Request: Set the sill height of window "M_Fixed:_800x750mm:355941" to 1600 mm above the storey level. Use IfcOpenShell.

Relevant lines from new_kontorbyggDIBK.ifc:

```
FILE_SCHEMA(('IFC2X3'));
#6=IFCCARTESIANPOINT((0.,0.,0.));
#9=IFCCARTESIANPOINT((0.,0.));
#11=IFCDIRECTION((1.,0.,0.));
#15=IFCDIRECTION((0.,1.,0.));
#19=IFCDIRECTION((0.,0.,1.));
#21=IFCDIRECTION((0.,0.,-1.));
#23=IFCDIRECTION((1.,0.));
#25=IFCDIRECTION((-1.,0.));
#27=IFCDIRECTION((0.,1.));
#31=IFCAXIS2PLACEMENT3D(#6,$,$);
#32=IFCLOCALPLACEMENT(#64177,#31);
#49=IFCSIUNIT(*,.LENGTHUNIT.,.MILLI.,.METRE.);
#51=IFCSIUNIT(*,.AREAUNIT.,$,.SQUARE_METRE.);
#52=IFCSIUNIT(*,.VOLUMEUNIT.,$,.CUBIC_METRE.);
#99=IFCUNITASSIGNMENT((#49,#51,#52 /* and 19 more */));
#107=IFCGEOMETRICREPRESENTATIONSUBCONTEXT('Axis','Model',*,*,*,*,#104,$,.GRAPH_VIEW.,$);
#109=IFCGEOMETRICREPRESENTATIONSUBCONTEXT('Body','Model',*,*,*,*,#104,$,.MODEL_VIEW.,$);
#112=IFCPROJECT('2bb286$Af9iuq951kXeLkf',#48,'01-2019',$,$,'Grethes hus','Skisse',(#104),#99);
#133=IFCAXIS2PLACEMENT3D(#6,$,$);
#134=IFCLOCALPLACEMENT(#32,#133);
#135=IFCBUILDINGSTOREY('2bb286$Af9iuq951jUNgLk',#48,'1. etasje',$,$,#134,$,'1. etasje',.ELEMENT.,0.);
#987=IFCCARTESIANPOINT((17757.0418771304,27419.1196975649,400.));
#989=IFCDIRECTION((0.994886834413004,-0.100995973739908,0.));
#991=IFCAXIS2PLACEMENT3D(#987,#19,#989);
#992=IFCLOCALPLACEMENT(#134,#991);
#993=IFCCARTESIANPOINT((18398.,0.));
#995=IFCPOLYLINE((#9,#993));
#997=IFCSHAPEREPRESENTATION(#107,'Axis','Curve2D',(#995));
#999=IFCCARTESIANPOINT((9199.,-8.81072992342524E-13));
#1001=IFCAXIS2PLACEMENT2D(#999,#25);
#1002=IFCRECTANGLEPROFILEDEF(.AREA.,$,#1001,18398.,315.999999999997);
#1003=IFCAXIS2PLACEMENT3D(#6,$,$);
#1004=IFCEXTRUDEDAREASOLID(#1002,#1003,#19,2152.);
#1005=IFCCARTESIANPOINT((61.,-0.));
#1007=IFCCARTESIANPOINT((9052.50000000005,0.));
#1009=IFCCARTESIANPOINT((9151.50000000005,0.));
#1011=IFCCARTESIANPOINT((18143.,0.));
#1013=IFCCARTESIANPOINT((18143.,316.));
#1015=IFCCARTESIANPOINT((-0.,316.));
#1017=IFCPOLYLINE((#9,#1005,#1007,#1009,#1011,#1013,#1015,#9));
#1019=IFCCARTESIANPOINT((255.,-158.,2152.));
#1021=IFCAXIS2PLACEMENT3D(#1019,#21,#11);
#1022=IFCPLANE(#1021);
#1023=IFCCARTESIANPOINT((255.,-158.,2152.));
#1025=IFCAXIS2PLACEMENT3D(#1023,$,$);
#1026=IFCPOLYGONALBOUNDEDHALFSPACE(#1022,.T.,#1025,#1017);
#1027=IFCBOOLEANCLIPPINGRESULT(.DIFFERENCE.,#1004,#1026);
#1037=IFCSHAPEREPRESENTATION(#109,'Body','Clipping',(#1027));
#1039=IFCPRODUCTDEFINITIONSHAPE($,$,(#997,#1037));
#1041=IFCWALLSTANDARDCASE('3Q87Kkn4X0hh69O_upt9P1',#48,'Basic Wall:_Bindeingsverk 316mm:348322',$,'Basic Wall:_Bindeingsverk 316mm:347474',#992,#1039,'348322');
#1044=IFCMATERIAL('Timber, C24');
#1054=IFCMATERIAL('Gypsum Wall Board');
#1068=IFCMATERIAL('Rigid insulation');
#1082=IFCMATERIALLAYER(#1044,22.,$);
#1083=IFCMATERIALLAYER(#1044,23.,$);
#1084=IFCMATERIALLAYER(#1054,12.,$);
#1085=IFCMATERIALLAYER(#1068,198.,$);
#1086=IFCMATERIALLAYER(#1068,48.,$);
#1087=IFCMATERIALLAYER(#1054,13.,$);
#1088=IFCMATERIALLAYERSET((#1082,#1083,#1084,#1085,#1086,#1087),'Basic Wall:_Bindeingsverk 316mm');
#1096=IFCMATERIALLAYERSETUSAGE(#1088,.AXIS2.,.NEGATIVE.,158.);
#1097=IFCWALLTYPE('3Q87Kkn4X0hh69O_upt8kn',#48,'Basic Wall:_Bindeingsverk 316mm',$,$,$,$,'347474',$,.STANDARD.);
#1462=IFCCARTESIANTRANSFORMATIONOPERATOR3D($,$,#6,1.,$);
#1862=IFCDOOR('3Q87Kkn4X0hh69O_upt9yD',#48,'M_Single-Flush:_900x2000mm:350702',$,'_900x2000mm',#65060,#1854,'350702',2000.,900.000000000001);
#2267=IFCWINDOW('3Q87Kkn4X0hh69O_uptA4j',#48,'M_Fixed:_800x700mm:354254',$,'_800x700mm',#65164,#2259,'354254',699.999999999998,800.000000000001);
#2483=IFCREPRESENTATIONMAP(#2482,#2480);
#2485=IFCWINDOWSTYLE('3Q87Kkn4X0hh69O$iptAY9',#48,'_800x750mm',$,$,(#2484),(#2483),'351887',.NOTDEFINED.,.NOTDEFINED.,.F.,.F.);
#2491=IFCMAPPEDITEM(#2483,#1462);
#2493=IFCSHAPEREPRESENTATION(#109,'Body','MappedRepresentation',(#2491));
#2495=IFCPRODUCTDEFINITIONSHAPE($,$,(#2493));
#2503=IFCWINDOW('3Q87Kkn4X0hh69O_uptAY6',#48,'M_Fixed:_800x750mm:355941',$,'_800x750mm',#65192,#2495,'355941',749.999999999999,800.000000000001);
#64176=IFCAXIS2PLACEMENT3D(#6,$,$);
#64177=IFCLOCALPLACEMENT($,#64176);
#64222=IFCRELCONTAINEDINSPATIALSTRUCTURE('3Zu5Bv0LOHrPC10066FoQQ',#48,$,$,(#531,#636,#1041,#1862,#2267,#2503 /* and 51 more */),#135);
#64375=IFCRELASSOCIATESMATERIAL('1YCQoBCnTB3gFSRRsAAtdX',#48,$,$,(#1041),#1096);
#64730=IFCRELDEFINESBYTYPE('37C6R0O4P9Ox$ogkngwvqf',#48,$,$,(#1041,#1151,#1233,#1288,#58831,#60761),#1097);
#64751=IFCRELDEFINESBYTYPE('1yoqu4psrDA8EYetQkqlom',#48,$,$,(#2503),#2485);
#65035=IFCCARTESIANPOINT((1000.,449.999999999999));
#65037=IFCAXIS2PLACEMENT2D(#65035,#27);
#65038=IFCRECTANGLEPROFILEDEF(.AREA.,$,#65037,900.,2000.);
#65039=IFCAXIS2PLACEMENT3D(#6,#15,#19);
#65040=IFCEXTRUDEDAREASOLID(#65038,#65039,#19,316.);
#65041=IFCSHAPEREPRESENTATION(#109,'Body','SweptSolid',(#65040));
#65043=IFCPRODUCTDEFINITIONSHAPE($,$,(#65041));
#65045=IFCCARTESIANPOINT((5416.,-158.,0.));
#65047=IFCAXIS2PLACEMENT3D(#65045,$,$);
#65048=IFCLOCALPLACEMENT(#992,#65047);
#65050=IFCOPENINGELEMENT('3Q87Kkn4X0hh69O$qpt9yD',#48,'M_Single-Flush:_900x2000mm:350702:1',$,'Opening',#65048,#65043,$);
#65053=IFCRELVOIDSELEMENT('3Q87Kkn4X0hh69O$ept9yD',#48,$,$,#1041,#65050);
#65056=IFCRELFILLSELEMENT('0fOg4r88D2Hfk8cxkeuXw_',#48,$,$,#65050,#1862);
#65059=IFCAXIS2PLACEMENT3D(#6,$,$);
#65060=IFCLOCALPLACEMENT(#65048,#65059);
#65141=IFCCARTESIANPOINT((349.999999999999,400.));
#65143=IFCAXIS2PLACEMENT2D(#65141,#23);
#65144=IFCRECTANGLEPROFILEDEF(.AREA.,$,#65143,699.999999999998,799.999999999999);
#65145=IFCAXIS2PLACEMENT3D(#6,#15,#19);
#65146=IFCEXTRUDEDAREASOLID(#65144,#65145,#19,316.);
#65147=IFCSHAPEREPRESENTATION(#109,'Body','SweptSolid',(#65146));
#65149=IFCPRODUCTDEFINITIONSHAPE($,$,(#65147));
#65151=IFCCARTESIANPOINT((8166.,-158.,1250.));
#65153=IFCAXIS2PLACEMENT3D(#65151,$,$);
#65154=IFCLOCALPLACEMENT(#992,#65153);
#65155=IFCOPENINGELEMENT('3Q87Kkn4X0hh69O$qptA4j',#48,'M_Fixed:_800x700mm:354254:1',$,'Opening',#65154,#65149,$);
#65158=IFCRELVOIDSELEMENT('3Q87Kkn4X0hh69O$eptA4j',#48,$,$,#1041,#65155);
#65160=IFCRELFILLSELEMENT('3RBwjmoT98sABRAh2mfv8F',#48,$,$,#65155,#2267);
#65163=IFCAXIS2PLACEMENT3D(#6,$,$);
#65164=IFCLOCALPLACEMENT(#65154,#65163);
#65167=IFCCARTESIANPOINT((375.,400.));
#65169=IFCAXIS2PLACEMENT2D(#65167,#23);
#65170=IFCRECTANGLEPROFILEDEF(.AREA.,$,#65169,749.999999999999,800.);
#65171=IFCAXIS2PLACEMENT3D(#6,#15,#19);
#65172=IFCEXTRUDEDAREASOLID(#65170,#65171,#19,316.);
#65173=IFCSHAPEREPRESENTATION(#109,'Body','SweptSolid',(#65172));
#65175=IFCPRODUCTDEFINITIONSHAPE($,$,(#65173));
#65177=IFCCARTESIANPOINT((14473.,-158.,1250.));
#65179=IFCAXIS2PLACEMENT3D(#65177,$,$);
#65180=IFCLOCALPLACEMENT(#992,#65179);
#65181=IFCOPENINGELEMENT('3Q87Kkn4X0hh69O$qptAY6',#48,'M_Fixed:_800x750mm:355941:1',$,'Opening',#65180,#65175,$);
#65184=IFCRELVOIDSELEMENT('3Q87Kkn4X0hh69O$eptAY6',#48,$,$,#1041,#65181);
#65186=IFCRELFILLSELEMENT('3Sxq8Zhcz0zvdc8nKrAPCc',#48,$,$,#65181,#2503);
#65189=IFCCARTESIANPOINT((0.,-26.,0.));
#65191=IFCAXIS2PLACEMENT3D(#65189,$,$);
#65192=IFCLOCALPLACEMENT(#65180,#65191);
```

```python
import numpy as np
import ifcopenshell
import ifcopenshell.api.geometry
import ifcopenshell.geom
import ifcopenshell.util.element
import ifcopenshell.util.placement
import ifcopenshell.util.shape
import ifcopenshell.util.unit

model = ifcopenshell.open("new_kontorbyggDIBK.ifc")
unit_scale = ifcopenshell.util.unit.calculate_unit_scale(model)

window = model.by_guid("3Q87Kkn4X0hh69O_uptAY6")
opening = window.FillsVoids[0].RelatingOpeningElement
storey = ifcopenshell.util.element.get_container(window, ifc_class="IfcBuildingStorey")
level = ifcopenshell.util.placement.get_local_placement(storey.ObjectPlacement)[2, 3]

# The opening's origin need not be at the sill, so measure its lowest point.
shape = ifcopenshell.geom.create_shape(ifcopenshell.geom.settings(), opening)
bottom = ifcopenshell.util.shape.get_shape_bottom_elevation(shape, shape.geometry) / unit_scale
dz = level + 1.6 / unit_scale - bottom

shift = np.array([0.0, 0.0, dz])
# The window is placed relative to its opening, so it follows when the opening moves.
matrix = ifcopenshell.util.placement.get_local_placement(opening.ObjectPlacement)
matrix[:3, 3] += shift
ifcopenshell.api.geometry.edit_object_placement(
    model, product=opening, matrix=matrix, is_si=False, should_transform_children=True
)

print(f"moved by {dz * unit_scale:+.3f} m")

model.write("new_kontorbyggDIBK_updated.ifc")
```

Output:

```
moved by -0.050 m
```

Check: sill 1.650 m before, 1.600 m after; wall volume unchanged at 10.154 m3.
